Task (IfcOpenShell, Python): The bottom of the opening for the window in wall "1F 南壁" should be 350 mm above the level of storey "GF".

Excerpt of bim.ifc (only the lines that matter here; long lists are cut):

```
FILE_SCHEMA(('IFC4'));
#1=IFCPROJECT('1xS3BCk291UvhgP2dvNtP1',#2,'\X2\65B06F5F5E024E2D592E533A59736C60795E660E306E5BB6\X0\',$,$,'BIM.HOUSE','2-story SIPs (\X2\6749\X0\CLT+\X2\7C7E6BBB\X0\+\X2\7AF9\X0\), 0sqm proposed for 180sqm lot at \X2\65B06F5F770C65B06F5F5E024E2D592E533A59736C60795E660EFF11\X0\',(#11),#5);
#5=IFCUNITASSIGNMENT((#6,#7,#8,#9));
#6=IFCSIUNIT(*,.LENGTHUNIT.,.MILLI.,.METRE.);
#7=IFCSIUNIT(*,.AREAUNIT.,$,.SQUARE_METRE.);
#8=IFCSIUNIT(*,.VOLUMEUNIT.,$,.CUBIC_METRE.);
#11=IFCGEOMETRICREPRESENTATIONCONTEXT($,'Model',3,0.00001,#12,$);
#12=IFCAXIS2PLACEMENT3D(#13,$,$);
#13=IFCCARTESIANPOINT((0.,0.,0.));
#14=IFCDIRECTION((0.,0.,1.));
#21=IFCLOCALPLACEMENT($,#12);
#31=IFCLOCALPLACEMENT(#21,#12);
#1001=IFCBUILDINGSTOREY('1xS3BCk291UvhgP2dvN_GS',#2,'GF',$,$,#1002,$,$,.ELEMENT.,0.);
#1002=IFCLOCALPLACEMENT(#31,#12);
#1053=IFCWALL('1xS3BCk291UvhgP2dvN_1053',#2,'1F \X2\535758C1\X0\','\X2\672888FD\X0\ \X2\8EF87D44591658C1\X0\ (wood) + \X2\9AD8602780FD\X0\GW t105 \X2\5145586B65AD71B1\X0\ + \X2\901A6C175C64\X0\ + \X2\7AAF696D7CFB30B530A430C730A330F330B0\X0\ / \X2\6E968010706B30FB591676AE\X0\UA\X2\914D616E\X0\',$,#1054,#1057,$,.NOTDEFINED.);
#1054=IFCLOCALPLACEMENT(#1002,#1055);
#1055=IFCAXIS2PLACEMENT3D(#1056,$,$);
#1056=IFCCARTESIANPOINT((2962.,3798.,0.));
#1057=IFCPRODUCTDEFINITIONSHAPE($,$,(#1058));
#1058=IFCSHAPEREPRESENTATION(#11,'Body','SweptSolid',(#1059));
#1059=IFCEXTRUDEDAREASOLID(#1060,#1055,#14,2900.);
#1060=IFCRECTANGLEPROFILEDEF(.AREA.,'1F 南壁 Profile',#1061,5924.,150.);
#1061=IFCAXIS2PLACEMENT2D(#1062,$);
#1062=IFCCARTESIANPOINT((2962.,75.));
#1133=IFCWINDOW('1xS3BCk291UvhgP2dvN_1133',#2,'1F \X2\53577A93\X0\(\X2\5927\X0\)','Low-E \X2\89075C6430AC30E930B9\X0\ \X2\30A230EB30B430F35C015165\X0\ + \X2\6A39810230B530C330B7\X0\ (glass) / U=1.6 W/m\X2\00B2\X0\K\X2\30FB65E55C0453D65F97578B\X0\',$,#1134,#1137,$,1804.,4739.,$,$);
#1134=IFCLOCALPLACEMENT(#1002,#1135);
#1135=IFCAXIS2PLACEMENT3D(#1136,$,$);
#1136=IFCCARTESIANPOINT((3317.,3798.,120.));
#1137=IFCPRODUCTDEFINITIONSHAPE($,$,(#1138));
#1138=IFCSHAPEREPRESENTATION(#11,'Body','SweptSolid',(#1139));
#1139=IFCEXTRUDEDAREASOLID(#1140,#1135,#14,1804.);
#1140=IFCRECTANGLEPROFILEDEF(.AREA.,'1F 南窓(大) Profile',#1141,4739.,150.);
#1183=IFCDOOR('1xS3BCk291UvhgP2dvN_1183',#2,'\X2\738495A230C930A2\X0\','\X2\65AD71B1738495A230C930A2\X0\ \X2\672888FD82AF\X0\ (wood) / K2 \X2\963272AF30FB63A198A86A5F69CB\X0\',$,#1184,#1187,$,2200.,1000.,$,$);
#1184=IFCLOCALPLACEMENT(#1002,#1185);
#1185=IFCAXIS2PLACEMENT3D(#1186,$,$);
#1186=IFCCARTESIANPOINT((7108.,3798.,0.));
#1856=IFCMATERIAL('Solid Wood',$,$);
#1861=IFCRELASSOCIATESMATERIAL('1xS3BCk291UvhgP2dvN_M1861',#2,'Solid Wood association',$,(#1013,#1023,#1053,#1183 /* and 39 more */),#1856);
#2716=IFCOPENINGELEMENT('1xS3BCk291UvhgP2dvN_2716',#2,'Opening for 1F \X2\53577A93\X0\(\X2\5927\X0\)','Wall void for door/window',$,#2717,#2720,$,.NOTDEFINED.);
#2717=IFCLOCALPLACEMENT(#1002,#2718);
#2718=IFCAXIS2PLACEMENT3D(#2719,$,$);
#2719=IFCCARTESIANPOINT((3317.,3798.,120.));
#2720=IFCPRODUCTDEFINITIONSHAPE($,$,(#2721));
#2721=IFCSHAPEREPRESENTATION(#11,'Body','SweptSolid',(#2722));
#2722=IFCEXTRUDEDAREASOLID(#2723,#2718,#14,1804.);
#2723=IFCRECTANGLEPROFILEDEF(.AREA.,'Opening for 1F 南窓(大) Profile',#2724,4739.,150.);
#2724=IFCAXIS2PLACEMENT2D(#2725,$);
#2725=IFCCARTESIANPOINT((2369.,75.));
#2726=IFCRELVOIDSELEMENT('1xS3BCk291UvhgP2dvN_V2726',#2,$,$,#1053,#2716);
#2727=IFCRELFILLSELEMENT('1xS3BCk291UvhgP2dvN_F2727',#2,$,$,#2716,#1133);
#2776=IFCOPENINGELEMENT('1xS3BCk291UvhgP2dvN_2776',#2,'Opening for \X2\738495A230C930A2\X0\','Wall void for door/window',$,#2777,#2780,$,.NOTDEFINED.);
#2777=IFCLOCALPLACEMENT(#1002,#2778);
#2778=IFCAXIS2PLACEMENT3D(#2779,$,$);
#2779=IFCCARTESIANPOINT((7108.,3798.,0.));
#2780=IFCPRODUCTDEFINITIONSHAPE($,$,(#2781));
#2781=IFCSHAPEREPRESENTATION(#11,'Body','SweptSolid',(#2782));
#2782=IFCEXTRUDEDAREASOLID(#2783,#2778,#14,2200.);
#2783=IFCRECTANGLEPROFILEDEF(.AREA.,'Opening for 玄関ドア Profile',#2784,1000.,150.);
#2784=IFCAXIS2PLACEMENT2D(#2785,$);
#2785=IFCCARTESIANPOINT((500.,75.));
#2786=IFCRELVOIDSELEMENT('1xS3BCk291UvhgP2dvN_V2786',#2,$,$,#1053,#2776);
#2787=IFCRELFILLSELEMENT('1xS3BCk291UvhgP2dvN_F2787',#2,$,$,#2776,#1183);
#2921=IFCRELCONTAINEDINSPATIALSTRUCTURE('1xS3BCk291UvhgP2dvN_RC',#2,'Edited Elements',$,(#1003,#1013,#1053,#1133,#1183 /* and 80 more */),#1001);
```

```python
import numpy as np
import ifcopenshell
import ifcopenshell.api.geometry
import ifcopenshell.geom
import ifcopenshell.util.element
import ifcopenshell.util.placement
import ifcopenshell.util.shape
import ifcopenshell.util.unit

model = ifcopenshell.open("bim.ifc")
unit_scale = ifcopenshell.util.unit.calculate_unit_scale(model)

window = model.by_id(1133)
opening = window.FillsVoids[0].RelatingOpeningElement
storey = ifcopenshell.util.element.get_container(window, ifc_class="IfcBuildingStorey")
level = ifcopenshell.util.placement.get_local_placement(storey.ObjectPlacement)[2, 3]

# The opening's origin need not be at the sill, so measure its lowest point.
shape = ifcopenshell.geom.create_shape(ifcopenshell.geom.settings(), opening)
bottom = ifcopenshell.util.shape.get_shape_bottom_elevation(shape, shape.geometry) / unit_scale
dz = level + 0.35 / unit_scale - bottom

shift = np.array([0.0, 0.0, dz])
# The window is not placed relative to its opening, so move both.
for product in (opening, window):
    matrix = ifcopenshell.util.placement.get_local_placement(product.ObjectPlacement)
    matrix[:3, 3] += shift
    ifcopenshell.api.geometry.edit_object_placement(model, product=product, matrix=matrix, is_si=False)

print(f"moved by {dz * unit_scale:+.3f} m")

model.write("bim_edited.ifc")
```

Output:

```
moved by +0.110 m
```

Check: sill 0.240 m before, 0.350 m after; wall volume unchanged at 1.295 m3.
